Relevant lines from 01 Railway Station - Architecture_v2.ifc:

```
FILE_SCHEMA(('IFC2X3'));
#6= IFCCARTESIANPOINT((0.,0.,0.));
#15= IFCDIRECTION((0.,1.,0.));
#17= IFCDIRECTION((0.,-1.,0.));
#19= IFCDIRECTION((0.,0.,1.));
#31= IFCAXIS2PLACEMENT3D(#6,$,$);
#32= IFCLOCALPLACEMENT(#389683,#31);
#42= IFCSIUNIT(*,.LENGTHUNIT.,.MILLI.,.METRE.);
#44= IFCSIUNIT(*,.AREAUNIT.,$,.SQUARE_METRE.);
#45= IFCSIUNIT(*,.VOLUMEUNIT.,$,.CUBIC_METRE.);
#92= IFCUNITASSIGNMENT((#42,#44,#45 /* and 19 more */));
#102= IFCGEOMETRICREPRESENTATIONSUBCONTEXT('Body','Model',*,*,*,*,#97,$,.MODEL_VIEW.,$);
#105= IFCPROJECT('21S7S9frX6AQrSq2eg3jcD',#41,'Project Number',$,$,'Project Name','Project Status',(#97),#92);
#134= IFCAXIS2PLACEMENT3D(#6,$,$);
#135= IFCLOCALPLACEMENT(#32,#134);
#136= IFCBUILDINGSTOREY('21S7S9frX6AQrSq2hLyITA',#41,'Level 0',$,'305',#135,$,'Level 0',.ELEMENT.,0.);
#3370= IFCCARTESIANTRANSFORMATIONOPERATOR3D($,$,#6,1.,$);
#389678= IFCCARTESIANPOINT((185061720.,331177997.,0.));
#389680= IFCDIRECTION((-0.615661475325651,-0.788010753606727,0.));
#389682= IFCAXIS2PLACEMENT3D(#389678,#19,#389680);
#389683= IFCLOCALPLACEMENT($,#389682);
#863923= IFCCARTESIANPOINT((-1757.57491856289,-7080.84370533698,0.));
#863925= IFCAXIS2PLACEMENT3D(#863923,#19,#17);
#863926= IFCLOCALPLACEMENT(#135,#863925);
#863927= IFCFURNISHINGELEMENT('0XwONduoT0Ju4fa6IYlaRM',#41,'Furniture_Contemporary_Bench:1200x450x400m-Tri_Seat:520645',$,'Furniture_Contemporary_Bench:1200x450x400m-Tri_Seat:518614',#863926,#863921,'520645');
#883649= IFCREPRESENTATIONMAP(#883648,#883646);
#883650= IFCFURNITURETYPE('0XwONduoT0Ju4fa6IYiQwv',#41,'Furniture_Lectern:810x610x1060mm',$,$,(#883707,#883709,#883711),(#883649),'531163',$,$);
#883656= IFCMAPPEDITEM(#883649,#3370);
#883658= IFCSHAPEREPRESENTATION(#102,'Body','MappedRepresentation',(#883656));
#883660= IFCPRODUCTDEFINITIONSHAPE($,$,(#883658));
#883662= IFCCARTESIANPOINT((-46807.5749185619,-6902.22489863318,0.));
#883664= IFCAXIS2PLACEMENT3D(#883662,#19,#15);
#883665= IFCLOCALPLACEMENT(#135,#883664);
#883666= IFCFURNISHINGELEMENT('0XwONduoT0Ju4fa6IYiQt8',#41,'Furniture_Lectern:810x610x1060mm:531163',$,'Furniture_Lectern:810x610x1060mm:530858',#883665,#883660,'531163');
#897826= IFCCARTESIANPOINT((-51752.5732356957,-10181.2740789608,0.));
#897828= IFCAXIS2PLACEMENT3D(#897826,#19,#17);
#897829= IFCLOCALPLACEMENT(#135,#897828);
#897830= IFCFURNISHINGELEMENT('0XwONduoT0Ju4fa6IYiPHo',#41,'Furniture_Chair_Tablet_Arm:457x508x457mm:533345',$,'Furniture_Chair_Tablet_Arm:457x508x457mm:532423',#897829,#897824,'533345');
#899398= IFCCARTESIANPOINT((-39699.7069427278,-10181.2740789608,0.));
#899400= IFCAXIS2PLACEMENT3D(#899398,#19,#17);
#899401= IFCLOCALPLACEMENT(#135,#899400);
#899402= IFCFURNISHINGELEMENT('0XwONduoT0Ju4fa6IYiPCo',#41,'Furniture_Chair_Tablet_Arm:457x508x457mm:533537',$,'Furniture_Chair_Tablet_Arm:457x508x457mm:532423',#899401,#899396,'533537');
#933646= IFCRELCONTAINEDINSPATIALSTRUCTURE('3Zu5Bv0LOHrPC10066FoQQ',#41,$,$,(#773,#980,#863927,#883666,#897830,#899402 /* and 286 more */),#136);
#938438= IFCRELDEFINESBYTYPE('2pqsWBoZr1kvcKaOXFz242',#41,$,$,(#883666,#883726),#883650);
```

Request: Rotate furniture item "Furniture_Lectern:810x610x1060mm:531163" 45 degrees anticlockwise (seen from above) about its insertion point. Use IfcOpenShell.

```python
import ifcopenshell
import ifcopenshell.api.geometry
import ifcopenshell.util.placement

model = ifcopenshell.open("01 Railway Station - Architecture_v2.ifc")

item = model.by_guid("0XwONduoT0Ju4fa6IYiQt8")
matrix = ifcopenshell.util.placement.get_local_placement(item.ObjectPlacement)
matrix = matrix @ ifcopenshell.util.placement.rotation(45, "Z")
ifcopenshell.api.geometry.edit_object_placement(model, product=item, matrix=matrix, is_si=False)

print(ifcopenshell.util.placement.get_local_placement(item.ObjectPlacement).round(3) + 0.0)

model.write("01 Railway Station - Architecture_v2_v2.ifc")
```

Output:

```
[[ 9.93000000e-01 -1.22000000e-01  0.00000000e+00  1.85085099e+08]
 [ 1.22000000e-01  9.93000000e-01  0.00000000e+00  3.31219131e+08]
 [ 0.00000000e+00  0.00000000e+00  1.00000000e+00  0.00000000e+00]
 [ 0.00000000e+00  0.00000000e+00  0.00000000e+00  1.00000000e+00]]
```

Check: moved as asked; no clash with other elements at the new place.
